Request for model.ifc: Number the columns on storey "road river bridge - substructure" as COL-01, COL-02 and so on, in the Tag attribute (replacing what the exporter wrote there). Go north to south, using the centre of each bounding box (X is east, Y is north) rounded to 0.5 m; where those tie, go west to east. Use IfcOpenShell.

First a look at what the model holds.

```python
import ifcopenshell
import ifcopenshell.util.element
import ifcopenshell.util.placement

model = ifcopenshell.open("model.ifc")
print(model.schema)
storey = next(s for s in model.by_type("IfcBuildingStorey") if s.Name == "road river bridge - substructure")
columns = [e for e in ifcopenshell.util.element.get_decomposition(storey) if e.is_a("IfcColumn")]
for e in sorted(columns, key=lambda e: e.id()):
    origin = ifcopenshell.util.placement.get_local_placement(e.ObjectPlacement)[:3, 3]
    print(e.id(), e.Tag, e.Name, origin.round(2) + 0.0, sep=" | ")
```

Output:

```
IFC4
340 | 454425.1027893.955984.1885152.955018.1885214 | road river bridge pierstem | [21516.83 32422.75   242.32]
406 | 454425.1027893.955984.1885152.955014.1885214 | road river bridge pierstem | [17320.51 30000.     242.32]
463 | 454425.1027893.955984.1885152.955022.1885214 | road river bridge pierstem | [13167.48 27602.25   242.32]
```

```python
import ifcopenshell
import ifcopenshell.geom
import ifcopenshell.util.element
import ifcopenshell.util.shape

model = ifcopenshell.open("model.ifc")
settings = ifcopenshell.geom.settings()
settings.set("use-world-coords", True)


def centre(element):
    shape = ifcopenshell.geom.create_shape(settings, element)
    return ifcopenshell.util.shape.get_bbox_centroid(shape.geometry)


storey = next(s for s in model.by_type("IfcBuildingStorey") if s.Name == "road river bridge - substructure")
columns = [e for e in ifcopenshell.util.element.get_decomposition(storey) if e.is_a("IfcColumn")]

# Insertion points can sit at a corner or the storey origin, so sort by the geometry (in metres).
centres = {e: centre(e) for e in columns}
columns.sort(key=lambda e: (-round(centres[e][1] / 0.5), centres[e][0]))

for i, e in enumerate(columns, start=1):
    number = f"COL-{i:02d}"
    e.Tag = number
    print(e.id(), number)

model.write("model_rev.ifc")
```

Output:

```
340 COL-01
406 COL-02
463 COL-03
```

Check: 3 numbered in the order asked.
